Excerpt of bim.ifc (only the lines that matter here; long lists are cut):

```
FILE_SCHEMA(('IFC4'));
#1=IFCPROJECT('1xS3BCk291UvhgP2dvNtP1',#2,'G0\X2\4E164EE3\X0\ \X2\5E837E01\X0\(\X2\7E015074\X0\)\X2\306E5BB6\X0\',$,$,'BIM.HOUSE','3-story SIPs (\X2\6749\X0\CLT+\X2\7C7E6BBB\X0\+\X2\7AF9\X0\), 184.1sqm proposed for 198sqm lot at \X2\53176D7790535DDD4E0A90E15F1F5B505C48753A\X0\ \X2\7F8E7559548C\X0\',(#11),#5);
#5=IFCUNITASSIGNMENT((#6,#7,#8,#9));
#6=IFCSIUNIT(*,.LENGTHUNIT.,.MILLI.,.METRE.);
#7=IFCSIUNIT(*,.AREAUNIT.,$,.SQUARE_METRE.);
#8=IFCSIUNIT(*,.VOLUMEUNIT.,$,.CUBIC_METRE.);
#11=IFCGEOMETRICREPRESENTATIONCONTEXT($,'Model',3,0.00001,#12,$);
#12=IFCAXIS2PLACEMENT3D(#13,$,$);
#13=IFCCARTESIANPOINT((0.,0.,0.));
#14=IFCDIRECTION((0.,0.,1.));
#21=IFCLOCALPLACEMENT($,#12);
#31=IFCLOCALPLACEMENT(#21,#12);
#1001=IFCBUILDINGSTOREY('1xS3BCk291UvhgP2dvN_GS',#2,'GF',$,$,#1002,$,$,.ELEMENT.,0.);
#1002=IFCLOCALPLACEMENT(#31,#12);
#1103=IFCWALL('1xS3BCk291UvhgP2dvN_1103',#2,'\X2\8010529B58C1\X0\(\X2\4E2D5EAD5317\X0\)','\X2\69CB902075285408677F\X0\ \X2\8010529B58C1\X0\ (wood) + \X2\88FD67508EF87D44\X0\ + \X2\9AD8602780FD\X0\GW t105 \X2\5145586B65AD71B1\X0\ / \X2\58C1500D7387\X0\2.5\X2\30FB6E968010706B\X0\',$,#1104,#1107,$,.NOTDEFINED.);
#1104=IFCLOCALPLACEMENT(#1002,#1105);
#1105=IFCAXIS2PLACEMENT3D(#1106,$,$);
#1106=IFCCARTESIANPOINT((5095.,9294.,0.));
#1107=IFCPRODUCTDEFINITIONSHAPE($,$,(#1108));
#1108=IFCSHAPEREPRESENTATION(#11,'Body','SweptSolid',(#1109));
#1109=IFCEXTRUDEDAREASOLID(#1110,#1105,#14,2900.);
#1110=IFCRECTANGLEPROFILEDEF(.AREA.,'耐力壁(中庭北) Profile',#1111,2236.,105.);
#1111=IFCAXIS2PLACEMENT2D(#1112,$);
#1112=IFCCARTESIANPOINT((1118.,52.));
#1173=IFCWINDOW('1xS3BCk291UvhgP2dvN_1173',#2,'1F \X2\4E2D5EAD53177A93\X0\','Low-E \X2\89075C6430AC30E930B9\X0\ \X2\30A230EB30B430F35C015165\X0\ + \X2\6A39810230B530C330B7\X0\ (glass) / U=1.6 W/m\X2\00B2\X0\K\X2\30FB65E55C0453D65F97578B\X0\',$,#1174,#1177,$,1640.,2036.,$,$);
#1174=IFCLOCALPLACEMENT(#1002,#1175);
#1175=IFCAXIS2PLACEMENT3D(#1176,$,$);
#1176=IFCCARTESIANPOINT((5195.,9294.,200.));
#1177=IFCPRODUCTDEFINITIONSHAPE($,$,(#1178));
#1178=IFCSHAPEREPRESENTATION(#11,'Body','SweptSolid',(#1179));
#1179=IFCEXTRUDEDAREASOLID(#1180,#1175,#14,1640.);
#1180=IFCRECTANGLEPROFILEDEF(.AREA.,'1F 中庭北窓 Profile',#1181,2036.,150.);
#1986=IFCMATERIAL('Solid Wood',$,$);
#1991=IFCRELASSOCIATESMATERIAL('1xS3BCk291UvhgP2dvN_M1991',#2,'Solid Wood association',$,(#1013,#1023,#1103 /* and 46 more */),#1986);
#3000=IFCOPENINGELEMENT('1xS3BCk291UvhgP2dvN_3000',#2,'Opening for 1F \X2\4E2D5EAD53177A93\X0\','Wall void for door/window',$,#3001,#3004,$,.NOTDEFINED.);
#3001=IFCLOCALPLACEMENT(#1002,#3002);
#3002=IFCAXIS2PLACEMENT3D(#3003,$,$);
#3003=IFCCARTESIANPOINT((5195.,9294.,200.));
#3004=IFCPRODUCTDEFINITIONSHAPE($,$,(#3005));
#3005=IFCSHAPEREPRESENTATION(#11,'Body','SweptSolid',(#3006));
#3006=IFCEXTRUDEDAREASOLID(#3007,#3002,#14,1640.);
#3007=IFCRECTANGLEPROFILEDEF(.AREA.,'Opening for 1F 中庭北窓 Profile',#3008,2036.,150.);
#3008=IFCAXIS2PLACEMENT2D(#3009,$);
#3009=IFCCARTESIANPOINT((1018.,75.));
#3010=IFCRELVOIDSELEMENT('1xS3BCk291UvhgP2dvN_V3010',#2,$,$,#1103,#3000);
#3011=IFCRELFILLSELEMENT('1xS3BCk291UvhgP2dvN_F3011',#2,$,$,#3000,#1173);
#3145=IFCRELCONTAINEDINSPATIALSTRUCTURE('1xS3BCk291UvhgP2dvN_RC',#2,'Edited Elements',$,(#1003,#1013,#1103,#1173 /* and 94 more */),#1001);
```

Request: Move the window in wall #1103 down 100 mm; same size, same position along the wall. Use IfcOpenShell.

```python
import numpy as np
import ifcopenshell
import ifcopenshell.api.geometry
import ifcopenshell.util.placement
import ifcopenshell.util.unit

model = ifcopenshell.open("bim.ifc")
unit_scale = ifcopenshell.util.unit.calculate_unit_scale(model)

window = model.by_guid("1xS3BCk291UvhgP2dvN_1173")
opening = window.FillsVoids[0].RelatingOpeningElement
dz = -0.1 / unit_scale

shift = np.array([0.0, 0.0, dz])
# The window is not placed relative to its opening, so move both.
for product in (opening, window):
    matrix = ifcopenshell.util.placement.get_local_placement(product.ObjectPlacement)
    matrix[:3, 3] += shift
    ifcopenshell.api.geometry.edit_object_placement(model, product=product, matrix=matrix, is_si=False)

print(f"moved by {dz * unit_scale:+.3f} m")

model.write("bim_updated.ifc")
```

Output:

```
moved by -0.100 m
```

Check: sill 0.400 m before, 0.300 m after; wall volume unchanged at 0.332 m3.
